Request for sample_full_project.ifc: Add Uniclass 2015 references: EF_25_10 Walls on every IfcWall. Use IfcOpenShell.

First a look at what the model holds.

```python
import ifcopenshell

model = ifcopenshell.open("sample_full_project.ifc")
print(model.schema)
print("classifications:", [c.Name for c in model.by_type("IfcClassification")])
for ifc_class in ("IfcDoor", "IfcRoof", "IfcStair", "IfcWall", "IfcWindow"):
    print(ifc_class, len(model.by_type(ifc_class)))
```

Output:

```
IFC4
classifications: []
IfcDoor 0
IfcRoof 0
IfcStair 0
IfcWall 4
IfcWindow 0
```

```python
import ifcopenshell
import ifcopenshell.api.classification

model = ifcopenshell.open("sample_full_project.ifc")

system = ifcopenshell.api.classification.add_classification(model, classification="Uniclass 2015")

codes = {
    "IfcWall": ("EF_25_10", "Walls"),
}
for ifc_class, (code, name) in codes.items():
    products = model.by_type(ifc_class)
    ifcopenshell.api.classification.add_reference(
        model, products=products, classification=system, identification=code, name=name
    )
    print(code, len(products))

model.write("sample_full_project_rev.ifc")
```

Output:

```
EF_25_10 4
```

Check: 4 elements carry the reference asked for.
